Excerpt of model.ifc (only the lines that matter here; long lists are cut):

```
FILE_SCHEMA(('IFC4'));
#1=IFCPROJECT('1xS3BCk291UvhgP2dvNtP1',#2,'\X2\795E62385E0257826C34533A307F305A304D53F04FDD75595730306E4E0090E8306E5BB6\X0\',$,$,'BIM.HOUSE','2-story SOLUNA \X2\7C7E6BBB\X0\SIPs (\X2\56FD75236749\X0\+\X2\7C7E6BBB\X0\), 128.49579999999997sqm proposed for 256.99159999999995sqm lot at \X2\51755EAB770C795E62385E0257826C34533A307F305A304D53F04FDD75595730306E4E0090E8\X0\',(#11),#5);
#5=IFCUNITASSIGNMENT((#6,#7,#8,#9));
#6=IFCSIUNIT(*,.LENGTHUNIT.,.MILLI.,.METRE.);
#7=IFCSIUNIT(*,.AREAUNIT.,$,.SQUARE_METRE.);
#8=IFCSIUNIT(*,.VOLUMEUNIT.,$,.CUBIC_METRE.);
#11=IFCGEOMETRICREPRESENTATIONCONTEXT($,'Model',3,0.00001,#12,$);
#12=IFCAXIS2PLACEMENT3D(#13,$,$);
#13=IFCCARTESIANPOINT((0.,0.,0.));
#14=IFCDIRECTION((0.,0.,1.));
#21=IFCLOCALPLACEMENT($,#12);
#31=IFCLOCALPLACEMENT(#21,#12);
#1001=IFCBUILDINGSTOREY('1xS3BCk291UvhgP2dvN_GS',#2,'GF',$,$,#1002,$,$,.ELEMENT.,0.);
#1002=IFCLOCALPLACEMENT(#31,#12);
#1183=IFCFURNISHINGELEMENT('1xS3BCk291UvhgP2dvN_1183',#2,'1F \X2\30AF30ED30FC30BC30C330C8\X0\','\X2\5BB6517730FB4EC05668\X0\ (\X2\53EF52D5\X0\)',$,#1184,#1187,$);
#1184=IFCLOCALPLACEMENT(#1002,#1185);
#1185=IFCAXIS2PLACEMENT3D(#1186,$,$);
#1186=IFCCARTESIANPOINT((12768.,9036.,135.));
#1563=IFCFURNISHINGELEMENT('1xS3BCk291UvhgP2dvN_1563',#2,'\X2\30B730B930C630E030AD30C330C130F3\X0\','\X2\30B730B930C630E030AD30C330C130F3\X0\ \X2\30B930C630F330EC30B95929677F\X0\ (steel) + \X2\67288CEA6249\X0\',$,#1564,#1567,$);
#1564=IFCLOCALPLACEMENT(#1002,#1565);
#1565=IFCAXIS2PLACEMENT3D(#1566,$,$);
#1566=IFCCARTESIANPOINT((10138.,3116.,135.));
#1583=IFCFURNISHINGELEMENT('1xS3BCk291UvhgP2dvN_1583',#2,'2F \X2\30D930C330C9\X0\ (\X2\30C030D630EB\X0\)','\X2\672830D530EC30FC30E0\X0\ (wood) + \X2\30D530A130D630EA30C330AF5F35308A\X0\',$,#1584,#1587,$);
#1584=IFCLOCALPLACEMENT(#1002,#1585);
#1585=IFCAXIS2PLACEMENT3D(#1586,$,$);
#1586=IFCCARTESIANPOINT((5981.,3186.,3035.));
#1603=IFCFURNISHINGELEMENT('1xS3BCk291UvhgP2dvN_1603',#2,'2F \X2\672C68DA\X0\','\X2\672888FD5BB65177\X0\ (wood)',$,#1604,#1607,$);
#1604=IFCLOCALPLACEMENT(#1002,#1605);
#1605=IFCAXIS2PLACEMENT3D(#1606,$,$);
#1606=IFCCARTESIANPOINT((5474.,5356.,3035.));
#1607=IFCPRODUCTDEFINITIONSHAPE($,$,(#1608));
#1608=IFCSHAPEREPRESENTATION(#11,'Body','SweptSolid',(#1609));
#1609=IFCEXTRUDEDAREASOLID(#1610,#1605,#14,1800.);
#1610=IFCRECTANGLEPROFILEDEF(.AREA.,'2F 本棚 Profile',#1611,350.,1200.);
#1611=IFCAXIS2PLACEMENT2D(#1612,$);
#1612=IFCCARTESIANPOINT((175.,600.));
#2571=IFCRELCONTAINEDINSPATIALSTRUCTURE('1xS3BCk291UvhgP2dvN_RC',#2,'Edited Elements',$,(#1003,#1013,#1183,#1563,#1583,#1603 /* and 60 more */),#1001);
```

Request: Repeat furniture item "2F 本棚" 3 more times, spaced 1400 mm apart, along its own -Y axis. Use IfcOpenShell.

```python
import ifcopenshell
import ifcopenshell.api.geometry
import ifcopenshell.api.root
import ifcopenshell.util.element
import ifcopenshell.util.placement
import ifcopenshell.util.unit

model = ifcopenshell.open("model.ifc")
unit_scale = ifcopenshell.util.unit.calculate_unit_scale(model)


def reuse_history(source, copy):
    """copy_class also copies each property set's owner history, people and application; keep the originals."""
    for rel in copy.IsDefinedBy:
        if rel.is_a("IfcRelDefinesByProperties") and (history := rel.RelatingPropertyDefinition.OwnerHistory):
            rel.RelatingPropertyDefinition.OwnerHistory = source.OwnerHistory
            ifcopenshell.util.element.remove_deep2(model, history)


source = model.by_guid("1xS3BCk291UvhgP2dvN_1603")
base = ifcopenshell.util.placement.get_local_placement(source.ObjectPlacement)
step = -base[:3, 1] * 1.4 / unit_scale

for i in range(1, 4):
    copy = ifcopenshell.api.root.copy_class(model, product=source)
    copy.Representation = ifcopenshell.util.element.copy_deep(
        model, source.Representation, exclude=["IfcGeometricRepresentationContext", "IfcRepresentationMap"]
    )
    reuse_history(source, copy)
    matrix = base.copy()
    matrix[:3, 3] += i * step
    print("added at", matrix[:3, 3].round(3) + 0.0)
    ifcopenshell.api.geometry.edit_object_placement(model, product=copy, matrix=matrix, is_si=False)

model.write("model-out.ifc")
```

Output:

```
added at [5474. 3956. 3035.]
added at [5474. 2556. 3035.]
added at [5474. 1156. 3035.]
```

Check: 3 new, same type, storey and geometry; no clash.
